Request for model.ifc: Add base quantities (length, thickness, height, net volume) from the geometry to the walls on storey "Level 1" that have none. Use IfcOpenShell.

First a look at what the model holds.

```python
import ifcopenshell
import ifcopenshell.util.element
import ifcopenshell.util.unit

model = ifcopenshell.open("model.ifc")
print(model.schema)
for unit_type in ("LENGTHUNIT", "AREAUNIT", "VOLUMEUNIT"):
    print(unit_type, ifcopenshell.util.unit.calculate_unit_scale(model, unit_type))
storey = next(s for s in model.by_type("IfcBuildingStorey") if s.Name == "Level 1")
walls = [e for e in ifcopenshell.util.element.get_decomposition(storey) if e.is_a("IfcWall")]
for e in sorted(walls, key=lambda e: e.id()):
    print(e.id(), e.is_a(), e.Name, list(ifcopenshell.util.element.get_psets(e, qtos_only=True)), sep=" | ")
```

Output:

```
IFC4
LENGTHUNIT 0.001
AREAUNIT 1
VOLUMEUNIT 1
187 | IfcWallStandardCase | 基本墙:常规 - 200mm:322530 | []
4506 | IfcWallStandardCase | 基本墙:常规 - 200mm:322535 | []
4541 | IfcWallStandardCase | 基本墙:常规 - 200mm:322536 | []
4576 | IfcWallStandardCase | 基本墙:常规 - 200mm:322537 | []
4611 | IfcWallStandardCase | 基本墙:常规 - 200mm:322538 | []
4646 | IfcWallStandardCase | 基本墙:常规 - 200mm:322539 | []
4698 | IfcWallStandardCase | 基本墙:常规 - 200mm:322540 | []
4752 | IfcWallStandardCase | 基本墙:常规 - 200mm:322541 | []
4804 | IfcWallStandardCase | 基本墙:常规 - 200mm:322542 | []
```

```python
import ifcopenshell
import ifcopenshell.api.pset
import ifcopenshell.geom
import ifcopenshell.util.element
import ifcopenshell.util.shape
import ifcopenshell.util.unit

model = ifcopenshell.open("model.ifc")
unit_scale = ifcopenshell.util.unit.calculate_unit_scale(model)
volume_scale = ifcopenshell.util.unit.calculate_unit_scale(model, "VOLUMEUNIT")
settings = ifcopenshell.geom.settings()

storey = next(s for s in model.by_type("IfcBuildingStorey") if s.Name == "Level 1")
walls = [e for e in ifcopenshell.util.element.get_decomposition(storey) if e.is_a("IfcWall")]

for e in sorted(walls, key=lambda e: e.id()):
    if ifcopenshell.util.element.get_psets(e, qtos_only=True, should_inherit=False):
        continue
    # Geometry comes back in metres, in the element's own axes.
    shape = ifcopenshell.geom.create_shape(settings, e)
    values = {
        "Length": ifcopenshell.util.shape.get_x(shape.geometry) / unit_scale,
        "Width": ifcopenshell.util.shape.get_y(shape.geometry) / unit_scale,
        "Height": ifcopenshell.util.shape.get_z(shape.geometry) / unit_scale,
        "NetVolume": ifcopenshell.util.shape.get_volume(shape.geometry) / volume_scale,
    }
    qto = ifcopenshell.api.pset.add_qto(model, product=e, name="Qto_WallBaseQuantities")
    ifcopenshell.api.pset.edit_qto(model, qto=qto, properties=values)
    print(e.id(), {k: round(v, 3) for k, v in values.items()})

model.write("model_v2.ifc")
```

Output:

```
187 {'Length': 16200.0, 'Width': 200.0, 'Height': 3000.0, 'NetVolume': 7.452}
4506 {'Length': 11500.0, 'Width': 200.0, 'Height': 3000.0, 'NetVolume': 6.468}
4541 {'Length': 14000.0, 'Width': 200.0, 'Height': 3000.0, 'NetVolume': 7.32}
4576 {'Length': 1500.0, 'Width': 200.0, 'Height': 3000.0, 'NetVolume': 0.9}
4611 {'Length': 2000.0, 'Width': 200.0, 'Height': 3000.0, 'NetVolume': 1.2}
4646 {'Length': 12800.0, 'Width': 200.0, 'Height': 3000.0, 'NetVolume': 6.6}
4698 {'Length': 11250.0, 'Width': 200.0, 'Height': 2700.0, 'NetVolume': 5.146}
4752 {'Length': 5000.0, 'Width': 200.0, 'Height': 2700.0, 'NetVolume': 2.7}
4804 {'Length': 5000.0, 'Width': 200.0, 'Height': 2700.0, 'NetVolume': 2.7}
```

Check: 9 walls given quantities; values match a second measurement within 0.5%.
